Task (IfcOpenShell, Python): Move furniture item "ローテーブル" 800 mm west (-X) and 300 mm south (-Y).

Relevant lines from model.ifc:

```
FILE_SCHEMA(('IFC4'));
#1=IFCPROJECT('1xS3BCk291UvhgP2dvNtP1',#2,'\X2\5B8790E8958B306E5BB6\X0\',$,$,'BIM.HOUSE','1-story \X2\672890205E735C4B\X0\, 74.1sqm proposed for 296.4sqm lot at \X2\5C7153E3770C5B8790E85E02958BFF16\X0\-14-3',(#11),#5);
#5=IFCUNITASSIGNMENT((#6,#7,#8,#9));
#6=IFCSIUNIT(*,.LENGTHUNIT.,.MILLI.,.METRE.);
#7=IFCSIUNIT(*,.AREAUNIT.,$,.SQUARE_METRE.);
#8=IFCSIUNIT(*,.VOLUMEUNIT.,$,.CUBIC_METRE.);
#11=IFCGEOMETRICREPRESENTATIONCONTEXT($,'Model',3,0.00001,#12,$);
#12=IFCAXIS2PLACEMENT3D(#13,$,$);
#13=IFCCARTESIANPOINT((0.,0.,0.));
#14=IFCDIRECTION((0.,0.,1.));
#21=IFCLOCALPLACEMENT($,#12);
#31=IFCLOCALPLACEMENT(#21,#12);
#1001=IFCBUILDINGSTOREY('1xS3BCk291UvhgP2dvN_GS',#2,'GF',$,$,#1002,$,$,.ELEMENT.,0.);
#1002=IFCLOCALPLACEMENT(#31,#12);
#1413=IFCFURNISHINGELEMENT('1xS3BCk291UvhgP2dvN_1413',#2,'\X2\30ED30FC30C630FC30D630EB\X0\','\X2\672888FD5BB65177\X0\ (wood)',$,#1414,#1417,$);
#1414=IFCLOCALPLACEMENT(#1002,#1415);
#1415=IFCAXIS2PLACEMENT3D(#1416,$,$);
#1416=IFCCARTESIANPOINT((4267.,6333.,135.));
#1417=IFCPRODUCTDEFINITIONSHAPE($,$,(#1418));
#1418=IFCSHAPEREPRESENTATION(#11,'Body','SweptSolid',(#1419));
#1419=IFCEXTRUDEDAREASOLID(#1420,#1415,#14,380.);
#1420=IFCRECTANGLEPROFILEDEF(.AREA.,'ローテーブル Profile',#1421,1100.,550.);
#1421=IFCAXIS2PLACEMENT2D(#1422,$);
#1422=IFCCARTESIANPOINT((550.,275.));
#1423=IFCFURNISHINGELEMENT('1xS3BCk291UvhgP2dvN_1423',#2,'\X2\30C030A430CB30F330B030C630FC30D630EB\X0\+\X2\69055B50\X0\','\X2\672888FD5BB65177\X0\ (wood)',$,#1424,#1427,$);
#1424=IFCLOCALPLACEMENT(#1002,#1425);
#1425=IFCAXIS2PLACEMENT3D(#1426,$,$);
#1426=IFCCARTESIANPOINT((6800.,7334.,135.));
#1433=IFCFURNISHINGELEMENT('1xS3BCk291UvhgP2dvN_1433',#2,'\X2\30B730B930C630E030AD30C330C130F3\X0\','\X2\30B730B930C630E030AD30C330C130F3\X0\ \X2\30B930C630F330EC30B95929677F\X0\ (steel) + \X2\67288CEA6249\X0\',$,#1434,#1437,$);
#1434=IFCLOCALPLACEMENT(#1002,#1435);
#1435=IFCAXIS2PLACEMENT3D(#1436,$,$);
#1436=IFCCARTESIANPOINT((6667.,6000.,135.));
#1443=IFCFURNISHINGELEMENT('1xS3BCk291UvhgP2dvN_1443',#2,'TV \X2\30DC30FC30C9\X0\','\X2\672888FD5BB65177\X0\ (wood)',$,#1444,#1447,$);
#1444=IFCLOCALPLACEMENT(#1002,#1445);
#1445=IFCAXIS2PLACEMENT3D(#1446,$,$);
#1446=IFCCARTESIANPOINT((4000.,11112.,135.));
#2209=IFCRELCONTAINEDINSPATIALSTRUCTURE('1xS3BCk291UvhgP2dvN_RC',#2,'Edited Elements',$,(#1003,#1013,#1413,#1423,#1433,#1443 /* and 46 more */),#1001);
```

```python
import ifcopenshell
import ifcopenshell.api.geometry
import ifcopenshell.util.placement
import ifcopenshell.util.unit

model = ifcopenshell.open("model.ifc")
unit_scale = ifcopenshell.util.unit.calculate_unit_scale(model)

item = model.by_id(1413)
matrix = ifcopenshell.util.placement.get_local_placement(item.ObjectPlacement)
matrix[0, 3] -= 0.8 / unit_scale
matrix[1, 3] -= 0.3 / unit_scale
ifcopenshell.api.geometry.edit_object_placement(model, product=item, matrix=matrix, is_si=False)

print(ifcopenshell.util.placement.get_local_placement(item.ObjectPlacement).round(3) + 0.0)

model.write("model_v2.ifc")
```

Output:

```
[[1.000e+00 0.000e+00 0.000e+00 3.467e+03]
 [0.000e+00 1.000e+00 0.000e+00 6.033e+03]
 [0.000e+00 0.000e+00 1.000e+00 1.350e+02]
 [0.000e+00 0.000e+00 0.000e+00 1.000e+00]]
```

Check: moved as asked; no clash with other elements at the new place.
